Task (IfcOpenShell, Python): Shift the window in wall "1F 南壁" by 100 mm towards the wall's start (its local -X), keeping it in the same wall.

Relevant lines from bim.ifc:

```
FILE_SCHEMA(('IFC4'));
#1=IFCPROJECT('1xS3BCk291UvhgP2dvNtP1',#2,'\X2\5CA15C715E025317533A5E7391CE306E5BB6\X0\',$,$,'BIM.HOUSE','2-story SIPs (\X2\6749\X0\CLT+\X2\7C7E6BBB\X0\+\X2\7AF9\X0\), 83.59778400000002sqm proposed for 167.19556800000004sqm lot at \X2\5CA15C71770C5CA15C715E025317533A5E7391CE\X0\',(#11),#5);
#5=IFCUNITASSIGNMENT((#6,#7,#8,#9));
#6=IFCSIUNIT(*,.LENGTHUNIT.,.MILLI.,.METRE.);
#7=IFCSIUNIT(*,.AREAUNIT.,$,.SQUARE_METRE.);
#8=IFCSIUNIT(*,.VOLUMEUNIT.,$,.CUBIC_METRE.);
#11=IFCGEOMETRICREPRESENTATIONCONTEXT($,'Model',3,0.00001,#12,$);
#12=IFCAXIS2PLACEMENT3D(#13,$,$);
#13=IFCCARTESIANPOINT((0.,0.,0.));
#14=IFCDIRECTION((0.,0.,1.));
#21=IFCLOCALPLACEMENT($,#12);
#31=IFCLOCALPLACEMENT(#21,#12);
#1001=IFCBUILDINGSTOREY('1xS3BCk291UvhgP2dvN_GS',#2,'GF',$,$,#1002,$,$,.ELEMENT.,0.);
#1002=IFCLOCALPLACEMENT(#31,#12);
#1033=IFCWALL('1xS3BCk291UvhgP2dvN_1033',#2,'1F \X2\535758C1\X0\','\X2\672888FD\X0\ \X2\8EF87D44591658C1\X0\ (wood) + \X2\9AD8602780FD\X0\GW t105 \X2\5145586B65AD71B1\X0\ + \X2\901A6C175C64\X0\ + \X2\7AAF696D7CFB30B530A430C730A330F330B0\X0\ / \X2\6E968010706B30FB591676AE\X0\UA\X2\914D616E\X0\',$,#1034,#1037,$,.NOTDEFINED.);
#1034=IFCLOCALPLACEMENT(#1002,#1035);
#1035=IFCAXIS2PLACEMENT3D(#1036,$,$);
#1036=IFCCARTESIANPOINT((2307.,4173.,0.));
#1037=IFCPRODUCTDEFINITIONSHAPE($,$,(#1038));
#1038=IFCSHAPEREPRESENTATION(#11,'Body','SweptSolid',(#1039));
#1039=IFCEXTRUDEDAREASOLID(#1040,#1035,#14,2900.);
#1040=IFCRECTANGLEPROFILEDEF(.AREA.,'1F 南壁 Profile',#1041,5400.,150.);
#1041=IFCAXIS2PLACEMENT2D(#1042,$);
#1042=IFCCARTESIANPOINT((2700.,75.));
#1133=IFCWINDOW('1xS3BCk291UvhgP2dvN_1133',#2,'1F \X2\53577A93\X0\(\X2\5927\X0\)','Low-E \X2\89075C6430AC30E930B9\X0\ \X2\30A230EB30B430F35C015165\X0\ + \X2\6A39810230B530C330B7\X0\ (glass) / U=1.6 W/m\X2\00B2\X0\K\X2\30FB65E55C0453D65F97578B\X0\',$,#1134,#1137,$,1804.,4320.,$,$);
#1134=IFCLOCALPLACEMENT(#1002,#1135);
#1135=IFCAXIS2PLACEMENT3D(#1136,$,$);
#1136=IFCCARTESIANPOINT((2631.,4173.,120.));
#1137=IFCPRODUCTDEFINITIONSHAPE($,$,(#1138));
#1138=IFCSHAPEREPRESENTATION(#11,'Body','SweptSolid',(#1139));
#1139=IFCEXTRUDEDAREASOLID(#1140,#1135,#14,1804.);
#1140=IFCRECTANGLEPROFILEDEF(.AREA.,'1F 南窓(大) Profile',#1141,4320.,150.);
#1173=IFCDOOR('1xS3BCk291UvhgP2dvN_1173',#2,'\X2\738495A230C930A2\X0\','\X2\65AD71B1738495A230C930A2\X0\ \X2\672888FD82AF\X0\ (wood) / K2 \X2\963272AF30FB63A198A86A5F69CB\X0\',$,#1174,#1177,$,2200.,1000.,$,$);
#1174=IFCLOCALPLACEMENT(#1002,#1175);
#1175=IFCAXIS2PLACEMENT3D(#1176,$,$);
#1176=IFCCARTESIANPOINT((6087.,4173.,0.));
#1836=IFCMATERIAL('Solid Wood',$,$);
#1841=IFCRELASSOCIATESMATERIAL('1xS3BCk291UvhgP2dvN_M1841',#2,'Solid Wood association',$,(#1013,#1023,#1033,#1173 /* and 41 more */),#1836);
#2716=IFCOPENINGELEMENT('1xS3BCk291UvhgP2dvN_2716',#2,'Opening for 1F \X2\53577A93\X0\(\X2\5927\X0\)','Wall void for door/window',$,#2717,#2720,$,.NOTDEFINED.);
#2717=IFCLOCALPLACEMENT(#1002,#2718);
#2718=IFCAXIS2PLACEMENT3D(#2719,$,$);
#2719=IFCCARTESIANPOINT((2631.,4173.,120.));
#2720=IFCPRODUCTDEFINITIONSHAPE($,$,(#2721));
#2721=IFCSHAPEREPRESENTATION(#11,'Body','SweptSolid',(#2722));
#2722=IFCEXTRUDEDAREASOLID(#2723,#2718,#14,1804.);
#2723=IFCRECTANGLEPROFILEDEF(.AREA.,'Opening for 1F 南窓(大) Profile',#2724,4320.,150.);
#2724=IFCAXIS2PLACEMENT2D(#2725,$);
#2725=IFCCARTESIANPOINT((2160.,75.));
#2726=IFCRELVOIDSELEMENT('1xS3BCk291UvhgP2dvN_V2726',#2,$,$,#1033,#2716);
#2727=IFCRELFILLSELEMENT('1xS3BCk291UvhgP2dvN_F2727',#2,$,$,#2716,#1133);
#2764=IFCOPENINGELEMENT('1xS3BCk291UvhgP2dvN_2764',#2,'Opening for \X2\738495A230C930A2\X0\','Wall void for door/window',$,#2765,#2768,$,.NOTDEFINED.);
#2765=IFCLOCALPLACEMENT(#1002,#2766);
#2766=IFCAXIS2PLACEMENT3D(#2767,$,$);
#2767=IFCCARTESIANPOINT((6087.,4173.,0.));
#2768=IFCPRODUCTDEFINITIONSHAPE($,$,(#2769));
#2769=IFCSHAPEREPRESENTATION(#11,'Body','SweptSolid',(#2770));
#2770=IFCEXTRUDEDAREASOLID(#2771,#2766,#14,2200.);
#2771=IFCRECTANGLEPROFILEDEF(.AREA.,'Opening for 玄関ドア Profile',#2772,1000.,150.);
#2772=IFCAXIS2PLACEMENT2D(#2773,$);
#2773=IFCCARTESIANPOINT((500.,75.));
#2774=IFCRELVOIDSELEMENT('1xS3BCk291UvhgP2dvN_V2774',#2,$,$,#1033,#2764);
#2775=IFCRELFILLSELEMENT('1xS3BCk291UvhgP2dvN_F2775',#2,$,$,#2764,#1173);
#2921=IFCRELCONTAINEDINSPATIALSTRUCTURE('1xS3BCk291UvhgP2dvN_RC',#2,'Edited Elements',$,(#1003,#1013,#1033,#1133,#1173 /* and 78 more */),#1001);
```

```python
import ifcopenshell
import ifcopenshell.api.geometry
import ifcopenshell.util.placement

model = ifcopenshell.open("bim.ifc")

window = model.by_guid("1xS3BCk291UvhgP2dvN_1133")
opening = window.FillsVoids[0].RelatingOpeningElement
wall = opening.VoidsElements[0].RelatingBuildingElement

wall_matrix = ifcopenshell.util.placement.get_local_placement(wall.ObjectPlacement)
shift = wall_matrix[:3, 0] * -100.0
before = ifcopenshell.util.placement.get_local_placement(window.ObjectPlacement)[:3, 3].copy()

# The window is not placed relative to its opening, so move both.
for product in (opening, window):
    matrix = ifcopenshell.util.placement.get_local_placement(product.ObjectPlacement)
    matrix[:3, 3] += shift
    ifcopenshell.api.geometry.edit_object_placement(model, product=product, matrix=matrix, is_si=False)

after = ifcopenshell.util.placement.get_local_placement(window.ObjectPlacement)[:3, 3]
print("window moved by", (after - before).round(3) + 0.0)

model.write("bim-out.ifc")
```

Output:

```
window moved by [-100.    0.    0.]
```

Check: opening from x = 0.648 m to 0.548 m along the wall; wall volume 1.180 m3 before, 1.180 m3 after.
